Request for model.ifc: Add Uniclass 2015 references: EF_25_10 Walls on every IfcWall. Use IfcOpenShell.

First a look at what the model holds.

```python
import ifcopenshell

model = ifcopenshell.open("model.ifc")
print(model.schema)
print("classifications:", [c.Name for c in model.by_type("IfcClassification")])
for ifc_class in ("IfcDoor", "IfcRoof", "IfcStair", "IfcWall", "IfcWindow"):
    print(ifc_class, len(model.by_type(ifc_class)))
```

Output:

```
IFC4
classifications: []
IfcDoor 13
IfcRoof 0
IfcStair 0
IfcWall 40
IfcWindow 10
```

```python
import ifcopenshell
import ifcopenshell.api.classification

model = ifcopenshell.open("model.ifc")

system = ifcopenshell.api.classification.add_classification(model, classification="Uniclass 2015")

codes = {
    "IfcWall": ("EF_25_10", "Walls"),
}
for ifc_class, (code, name) in codes.items():
    products = model.by_type(ifc_class)
    ifcopenshell.api.classification.add_reference(
        model, products=products, classification=system, identification=code, name=name
    )
    print(code, len(products))

model.write("model_rev.ifc")
```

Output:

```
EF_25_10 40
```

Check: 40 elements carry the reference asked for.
